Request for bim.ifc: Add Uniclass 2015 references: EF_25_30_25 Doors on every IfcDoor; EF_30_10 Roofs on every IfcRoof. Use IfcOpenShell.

First a look at what the model holds.

```python
import ifcopenshell

model = ifcopenshell.open("bim.ifc")
print(model.schema)
print("classifications:", [c.Name for c in model.by_type("IfcClassification")])
for ifc_class in ("IfcDoor", "IfcRoof", "IfcStair", "IfcWall", "IfcWindow"):
    print(ifc_class, len(model.by_type(ifc_class)))
```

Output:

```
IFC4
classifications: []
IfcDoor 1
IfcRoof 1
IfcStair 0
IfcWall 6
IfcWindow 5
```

```python
import ifcopenshell
import ifcopenshell.api.classification

model = ifcopenshell.open("bim.ifc")

system = ifcopenshell.api.classification.add_classification(model, classification="Uniclass 2015")

codes = {
    "IfcDoor": ("EF_25_30_25", "Doors"),
    "IfcRoof": ("EF_30_10", "Roofs"),
}
for ifc_class, (code, name) in codes.items():
    products = model.by_type(ifc_class)
    ifcopenshell.api.classification.add_reference(
        model, products=products, classification=system, identification=code, name=name
    )
    print(code, len(products))

model.write("bim_updated.ifc")
```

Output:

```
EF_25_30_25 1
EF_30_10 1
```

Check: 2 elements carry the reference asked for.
